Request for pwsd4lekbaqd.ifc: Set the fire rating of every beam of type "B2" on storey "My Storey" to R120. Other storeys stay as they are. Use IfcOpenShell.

First a look at what the model holds.

```python
import ifcopenshell
import ifcopenshell.util.element

model = ifcopenshell.open("pwsd4lekbaqd.ifc")
print(model.schema)
storey = next(s for s in model.by_type("IfcBuildingStorey") if s.Name == "My Storey")
beams = [e for e in ifcopenshell.util.element.get_decomposition(storey) if e.is_a("IfcBeam")]
seen = {}
for e in beams:
    element_type = ifcopenshell.util.element.get_type(e)
    key = (element_type.Name if element_type != e and element_type else None, ifcopenshell.util.element.get_pset(e, "Pset_BeamCommon", "FireRating"))
    seen[key] = seen.get(key, 0) + 1
for (name, value), count in sorted(seen.items(), key=str):
    print(count, "x", name, "|", value)
```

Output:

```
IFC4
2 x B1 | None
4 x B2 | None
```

```python
import ifcopenshell
import ifcopenshell.api.pset
import ifcopenshell.util.element

model = ifcopenshell.open("pwsd4lekbaqd.ifc")

storey = next(s for s in model.by_type("IfcBuildingStorey") if s.Name == "My Storey")
beams = [e for e in ifcopenshell.util.element.get_decomposition(storey) if e.is_a("IfcBeam")]

count = 0
for e in beams:
    element_type = ifcopenshell.util.element.get_type(e)
    if element_type in (None, e) or element_type.Name != "B2":
        continue
    # add_pset returns the element's existing set when there is one.
    pset = ifcopenshell.api.pset.add_pset(model, product=e, name="Pset_BeamCommon")
    ifcopenshell.api.pset.edit_pset(model, pset=pset, properties={"FireRating": "R120"})
    count += 1

print(count, "beams updated")

model.write("pwsd4lekbaqd_v2.ifc")
```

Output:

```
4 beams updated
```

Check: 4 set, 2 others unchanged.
